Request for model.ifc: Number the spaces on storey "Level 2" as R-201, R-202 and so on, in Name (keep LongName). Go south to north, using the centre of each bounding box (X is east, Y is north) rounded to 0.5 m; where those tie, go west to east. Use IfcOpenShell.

First a look at what the model holds.

```python
import ifcopenshell
import ifcopenshell.util.element
import ifcopenshell.util.placement

model = ifcopenshell.open("model.ifc")
print(model.schema)
storey = next(s for s in model.by_type("IfcBuildingStorey") if s.Name == "Level 2")
spaces = [e for e in ifcopenshell.util.element.get_decomposition(storey) if e.is_a("IfcSpace")]
for e in sorted(spaces, key=lambda e: e.id()):
    origin = ifcopenshell.util.placement.get_local_placement(e.ObjectPlacement)[:3, 3]
    print(e.id(), e.Name, e.LongName, origin.round(2) + 0.0, sep=" | ")
```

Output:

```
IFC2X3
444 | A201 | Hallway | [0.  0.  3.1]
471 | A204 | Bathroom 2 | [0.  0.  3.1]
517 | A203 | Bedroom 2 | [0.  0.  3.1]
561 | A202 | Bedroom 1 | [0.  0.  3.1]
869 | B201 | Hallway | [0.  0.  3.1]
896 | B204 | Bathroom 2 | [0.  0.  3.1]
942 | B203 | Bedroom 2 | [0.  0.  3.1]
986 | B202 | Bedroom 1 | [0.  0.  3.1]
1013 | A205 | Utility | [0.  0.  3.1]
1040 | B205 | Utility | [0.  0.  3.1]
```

```python
import ifcopenshell
import ifcopenshell.geom
import ifcopenshell.util.element
import ifcopenshell.util.shape

model = ifcopenshell.open("model.ifc")
settings = ifcopenshell.geom.settings()
settings.set("use-world-coords", True)


def centre(element):
    shape = ifcopenshell.geom.create_shape(settings, element)
    return ifcopenshell.util.shape.get_bbox_centroid(shape.geometry)


storey = next(s for s in model.by_type("IfcBuildingStorey") if s.Name == "Level 2")
spaces = [e for e in ifcopenshell.util.element.get_decomposition(storey) if e.is_a("IfcSpace")]

# Insertion points can sit at a corner or the storey origin, so sort by the geometry (in metres).
centres = {e: centre(e) for e in spaces}
spaces.sort(key=lambda e: (round(centres[e][1] / 0.5), centres[e][0]))

for i, e in enumerate(spaces, start=1):
    number = f"R-2{i:02d}"
    e.Name = number
    print(e.id(), number)

model.write("model_rev.ifc")
```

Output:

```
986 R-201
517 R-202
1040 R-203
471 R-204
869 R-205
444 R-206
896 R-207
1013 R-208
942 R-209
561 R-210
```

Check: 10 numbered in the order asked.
